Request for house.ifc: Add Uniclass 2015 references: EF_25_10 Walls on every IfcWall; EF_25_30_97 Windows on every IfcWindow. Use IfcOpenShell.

First a look at what the model holds.

```python
import ifcopenshell

model = ifcopenshell.open("house.ifc")
print(model.schema)
print("classifications:", [c.Name for c in model.by_type("IfcClassification")])
for ifc_class in ("IfcDoor", "IfcRoof", "IfcStair", "IfcWall", "IfcWindow"):
    print(ifc_class, len(model.by_type(ifc_class)))
```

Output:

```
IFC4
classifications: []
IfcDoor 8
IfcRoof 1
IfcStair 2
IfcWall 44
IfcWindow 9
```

```python
import ifcopenshell
import ifcopenshell.api.classification

model = ifcopenshell.open("house.ifc")

system = ifcopenshell.api.classification.add_classification(model, classification="Uniclass 2015")

codes = {
    "IfcWall": ("EF_25_10", "Walls"),
    "IfcWindow": ("EF_25_30_97", "Windows"),
}
for ifc_class, (code, name) in codes.items():
    products = model.by_type(ifc_class)
    ifcopenshell.api.classification.add_reference(
        model, products=products, classification=system, identification=code, name=name
    )
    print(code, len(products))

model.write("house-out.ifc")
```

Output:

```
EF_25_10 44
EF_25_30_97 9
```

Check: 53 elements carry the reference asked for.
